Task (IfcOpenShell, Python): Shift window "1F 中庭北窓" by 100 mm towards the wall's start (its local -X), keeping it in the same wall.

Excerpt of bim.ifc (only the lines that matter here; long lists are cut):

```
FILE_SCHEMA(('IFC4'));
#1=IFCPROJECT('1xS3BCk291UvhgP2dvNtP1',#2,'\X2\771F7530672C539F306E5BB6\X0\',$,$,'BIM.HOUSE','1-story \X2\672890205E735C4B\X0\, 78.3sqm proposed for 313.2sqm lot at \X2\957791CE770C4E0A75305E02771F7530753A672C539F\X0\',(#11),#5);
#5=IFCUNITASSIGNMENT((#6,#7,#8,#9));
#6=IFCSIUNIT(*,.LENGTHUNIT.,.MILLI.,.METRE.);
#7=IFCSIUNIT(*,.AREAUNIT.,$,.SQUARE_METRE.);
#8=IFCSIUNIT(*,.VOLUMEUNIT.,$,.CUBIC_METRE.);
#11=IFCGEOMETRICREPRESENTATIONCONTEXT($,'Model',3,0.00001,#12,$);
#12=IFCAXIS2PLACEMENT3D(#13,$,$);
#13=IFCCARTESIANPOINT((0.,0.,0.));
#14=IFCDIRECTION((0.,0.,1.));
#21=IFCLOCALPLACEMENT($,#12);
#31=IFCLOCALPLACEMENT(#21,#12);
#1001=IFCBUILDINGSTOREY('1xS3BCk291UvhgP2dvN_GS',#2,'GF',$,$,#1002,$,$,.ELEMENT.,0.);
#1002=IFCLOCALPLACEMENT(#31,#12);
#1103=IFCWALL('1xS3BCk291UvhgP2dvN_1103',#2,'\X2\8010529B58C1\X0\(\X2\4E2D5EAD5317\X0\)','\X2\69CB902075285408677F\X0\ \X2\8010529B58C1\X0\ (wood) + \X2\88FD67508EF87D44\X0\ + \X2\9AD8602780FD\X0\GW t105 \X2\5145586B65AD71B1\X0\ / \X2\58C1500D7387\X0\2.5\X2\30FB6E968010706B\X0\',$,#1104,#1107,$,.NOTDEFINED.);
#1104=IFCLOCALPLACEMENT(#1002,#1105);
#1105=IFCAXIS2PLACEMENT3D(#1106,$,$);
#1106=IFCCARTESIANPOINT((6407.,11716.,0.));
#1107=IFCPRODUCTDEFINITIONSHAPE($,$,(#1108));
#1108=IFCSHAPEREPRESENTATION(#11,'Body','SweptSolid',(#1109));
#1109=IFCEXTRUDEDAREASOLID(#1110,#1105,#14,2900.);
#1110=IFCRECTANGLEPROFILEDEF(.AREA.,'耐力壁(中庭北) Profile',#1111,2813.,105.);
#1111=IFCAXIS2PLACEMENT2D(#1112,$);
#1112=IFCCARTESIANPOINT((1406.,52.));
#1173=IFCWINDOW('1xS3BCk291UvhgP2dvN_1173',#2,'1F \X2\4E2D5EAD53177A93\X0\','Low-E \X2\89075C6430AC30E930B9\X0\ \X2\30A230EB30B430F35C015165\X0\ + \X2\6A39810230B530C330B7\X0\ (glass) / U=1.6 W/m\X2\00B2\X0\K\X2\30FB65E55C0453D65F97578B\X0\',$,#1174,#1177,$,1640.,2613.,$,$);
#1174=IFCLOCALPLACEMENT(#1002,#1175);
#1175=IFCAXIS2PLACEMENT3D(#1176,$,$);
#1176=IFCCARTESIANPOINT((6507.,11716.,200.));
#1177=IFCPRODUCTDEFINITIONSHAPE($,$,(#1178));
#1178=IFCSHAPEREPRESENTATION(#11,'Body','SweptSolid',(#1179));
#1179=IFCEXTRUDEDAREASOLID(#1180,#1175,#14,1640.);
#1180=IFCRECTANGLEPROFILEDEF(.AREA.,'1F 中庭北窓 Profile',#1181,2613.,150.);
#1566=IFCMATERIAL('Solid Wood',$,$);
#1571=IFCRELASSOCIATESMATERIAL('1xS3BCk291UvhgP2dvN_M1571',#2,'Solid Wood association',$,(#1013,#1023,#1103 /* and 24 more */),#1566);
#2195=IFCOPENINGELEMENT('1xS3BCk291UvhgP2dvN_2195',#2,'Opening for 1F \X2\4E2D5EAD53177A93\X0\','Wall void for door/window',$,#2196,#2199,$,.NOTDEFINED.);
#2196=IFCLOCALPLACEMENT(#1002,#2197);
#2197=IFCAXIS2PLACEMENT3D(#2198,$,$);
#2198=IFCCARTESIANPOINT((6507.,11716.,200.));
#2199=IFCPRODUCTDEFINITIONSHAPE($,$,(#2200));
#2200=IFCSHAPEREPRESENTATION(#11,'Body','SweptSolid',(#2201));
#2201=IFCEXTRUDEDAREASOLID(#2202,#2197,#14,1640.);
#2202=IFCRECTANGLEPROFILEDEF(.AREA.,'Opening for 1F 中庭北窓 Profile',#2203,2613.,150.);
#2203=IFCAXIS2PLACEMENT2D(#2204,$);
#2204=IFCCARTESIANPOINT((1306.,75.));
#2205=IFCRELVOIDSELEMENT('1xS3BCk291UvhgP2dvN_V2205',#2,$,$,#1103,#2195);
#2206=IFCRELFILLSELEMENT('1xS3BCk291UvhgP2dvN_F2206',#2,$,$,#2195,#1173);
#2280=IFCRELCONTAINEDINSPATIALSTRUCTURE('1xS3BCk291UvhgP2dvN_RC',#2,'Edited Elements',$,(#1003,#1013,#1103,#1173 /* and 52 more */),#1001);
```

```python
import ifcopenshell
import ifcopenshell.api.geometry
import ifcopenshell.util.placement
import ifcopenshell.util.unit

model = ifcopenshell.open("bim.ifc")
unit_scale = ifcopenshell.util.unit.calculate_unit_scale(model)

window = model.by_id(1173)
opening = window.FillsVoids[0].RelatingOpeningElement
wall = opening.VoidsElements[0].RelatingBuildingElement

wall_matrix = ifcopenshell.util.placement.get_local_placement(wall.ObjectPlacement)
shift = wall_matrix[:3, 0] * -0.1 / unit_scale
before = ifcopenshell.util.placement.get_local_placement(window.ObjectPlacement)[:3, 3].copy()

# The window is not placed relative to its opening, so move both.
for product in (opening, window):
    matrix = ifcopenshell.util.placement.get_local_placement(product.ObjectPlacement)
    matrix[:3, 3] += shift
    ifcopenshell.api.geometry.edit_object_placement(model, product=product, matrix=matrix, is_si=False)

after = ifcopenshell.util.placement.get_local_placement(window.ObjectPlacement)[:3, 3]
print("window moved by", (after - before).round(3) + 0.0)

model.write("bim-out.ifc")
```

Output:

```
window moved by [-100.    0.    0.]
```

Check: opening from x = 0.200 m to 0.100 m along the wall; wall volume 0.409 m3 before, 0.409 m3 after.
